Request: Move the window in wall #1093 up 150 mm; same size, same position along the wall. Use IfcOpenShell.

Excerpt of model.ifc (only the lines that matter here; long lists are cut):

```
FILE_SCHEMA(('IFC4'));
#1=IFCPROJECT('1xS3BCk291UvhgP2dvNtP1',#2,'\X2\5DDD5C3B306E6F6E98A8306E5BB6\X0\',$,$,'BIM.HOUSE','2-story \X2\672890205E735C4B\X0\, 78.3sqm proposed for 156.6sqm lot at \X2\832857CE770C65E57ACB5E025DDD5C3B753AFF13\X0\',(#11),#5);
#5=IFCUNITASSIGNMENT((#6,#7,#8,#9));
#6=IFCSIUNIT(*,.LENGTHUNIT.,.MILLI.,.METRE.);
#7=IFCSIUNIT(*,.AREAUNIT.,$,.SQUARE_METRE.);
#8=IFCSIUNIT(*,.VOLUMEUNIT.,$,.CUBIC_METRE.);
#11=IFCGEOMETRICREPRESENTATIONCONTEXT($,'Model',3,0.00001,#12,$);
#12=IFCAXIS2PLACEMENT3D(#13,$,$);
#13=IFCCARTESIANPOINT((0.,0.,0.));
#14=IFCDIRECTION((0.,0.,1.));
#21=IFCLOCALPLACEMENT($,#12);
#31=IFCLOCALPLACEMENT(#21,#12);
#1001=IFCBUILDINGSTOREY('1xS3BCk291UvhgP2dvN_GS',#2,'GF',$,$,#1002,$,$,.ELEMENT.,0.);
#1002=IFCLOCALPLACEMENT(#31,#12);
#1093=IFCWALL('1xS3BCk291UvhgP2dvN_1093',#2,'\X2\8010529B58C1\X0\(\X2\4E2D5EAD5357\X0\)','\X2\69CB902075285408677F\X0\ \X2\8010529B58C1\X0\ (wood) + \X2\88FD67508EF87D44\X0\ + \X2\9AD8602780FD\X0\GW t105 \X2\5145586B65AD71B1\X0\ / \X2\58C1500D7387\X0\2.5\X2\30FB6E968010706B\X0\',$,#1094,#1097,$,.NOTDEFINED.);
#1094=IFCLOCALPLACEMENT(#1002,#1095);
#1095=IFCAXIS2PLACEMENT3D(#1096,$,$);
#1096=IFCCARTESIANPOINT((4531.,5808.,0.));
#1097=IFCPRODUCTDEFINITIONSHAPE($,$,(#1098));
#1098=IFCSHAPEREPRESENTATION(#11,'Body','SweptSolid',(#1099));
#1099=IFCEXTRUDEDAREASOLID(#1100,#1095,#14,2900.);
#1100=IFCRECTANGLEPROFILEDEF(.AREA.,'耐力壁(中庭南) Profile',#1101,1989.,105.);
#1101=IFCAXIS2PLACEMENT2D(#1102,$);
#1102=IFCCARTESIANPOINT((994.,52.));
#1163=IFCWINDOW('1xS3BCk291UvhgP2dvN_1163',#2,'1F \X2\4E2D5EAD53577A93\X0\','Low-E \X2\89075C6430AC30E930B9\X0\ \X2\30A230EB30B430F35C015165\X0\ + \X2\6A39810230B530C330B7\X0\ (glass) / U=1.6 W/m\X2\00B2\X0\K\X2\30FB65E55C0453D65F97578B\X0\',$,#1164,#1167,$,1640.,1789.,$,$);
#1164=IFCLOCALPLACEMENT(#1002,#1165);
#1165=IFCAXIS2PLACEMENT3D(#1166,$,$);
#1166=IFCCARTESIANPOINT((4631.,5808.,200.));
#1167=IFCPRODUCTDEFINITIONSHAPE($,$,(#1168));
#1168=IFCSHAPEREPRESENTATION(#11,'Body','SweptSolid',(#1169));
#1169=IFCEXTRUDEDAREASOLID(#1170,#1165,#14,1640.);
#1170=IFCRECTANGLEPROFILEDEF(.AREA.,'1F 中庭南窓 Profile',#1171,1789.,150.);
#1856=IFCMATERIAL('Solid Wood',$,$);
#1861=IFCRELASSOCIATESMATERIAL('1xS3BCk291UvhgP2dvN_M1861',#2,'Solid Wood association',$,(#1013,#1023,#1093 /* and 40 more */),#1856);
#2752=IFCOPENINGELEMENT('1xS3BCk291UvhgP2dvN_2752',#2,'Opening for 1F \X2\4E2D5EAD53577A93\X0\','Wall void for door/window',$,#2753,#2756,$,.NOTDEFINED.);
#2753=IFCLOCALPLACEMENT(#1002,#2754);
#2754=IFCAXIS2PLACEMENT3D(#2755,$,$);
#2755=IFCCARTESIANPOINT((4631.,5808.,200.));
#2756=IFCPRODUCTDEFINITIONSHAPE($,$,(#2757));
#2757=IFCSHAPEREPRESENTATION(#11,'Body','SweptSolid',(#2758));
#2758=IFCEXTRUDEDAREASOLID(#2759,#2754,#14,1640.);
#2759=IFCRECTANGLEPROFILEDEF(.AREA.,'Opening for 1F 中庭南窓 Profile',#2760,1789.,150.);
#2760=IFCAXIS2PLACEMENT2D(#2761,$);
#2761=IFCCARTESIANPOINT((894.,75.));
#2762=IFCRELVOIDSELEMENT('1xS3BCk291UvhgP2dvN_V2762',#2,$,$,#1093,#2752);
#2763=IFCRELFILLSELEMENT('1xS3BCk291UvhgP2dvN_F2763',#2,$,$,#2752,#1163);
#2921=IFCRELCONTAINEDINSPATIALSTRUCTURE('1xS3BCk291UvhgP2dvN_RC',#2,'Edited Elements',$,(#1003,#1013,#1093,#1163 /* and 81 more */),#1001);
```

```python
import numpy as np
import ifcopenshell
import ifcopenshell.api.geometry
import ifcopenshell.util.placement
import ifcopenshell.util.unit

model = ifcopenshell.open("model.ifc")
unit_scale = ifcopenshell.util.unit.calculate_unit_scale(model)

window = model.by_guid("1xS3BCk291UvhgP2dvN_1163")
opening = window.FillsVoids[0].RelatingOpeningElement
dz = 0.15 / unit_scale

shift = np.array([0.0, 0.0, dz])
# The window is not placed relative to its opening, so move both.
for product in (opening, window):
    matrix = ifcopenshell.util.placement.get_local_placement(product.ObjectPlacement)
    matrix[:3, 3] += shift
    ifcopenshell.api.geometry.edit_object_placement(model, product=product, matrix=matrix, is_si=False)

print(f"moved by {dz * unit_scale:+.3f} m")

model.write("model_edited.ifc")
```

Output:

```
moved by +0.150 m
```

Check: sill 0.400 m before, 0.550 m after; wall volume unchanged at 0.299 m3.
